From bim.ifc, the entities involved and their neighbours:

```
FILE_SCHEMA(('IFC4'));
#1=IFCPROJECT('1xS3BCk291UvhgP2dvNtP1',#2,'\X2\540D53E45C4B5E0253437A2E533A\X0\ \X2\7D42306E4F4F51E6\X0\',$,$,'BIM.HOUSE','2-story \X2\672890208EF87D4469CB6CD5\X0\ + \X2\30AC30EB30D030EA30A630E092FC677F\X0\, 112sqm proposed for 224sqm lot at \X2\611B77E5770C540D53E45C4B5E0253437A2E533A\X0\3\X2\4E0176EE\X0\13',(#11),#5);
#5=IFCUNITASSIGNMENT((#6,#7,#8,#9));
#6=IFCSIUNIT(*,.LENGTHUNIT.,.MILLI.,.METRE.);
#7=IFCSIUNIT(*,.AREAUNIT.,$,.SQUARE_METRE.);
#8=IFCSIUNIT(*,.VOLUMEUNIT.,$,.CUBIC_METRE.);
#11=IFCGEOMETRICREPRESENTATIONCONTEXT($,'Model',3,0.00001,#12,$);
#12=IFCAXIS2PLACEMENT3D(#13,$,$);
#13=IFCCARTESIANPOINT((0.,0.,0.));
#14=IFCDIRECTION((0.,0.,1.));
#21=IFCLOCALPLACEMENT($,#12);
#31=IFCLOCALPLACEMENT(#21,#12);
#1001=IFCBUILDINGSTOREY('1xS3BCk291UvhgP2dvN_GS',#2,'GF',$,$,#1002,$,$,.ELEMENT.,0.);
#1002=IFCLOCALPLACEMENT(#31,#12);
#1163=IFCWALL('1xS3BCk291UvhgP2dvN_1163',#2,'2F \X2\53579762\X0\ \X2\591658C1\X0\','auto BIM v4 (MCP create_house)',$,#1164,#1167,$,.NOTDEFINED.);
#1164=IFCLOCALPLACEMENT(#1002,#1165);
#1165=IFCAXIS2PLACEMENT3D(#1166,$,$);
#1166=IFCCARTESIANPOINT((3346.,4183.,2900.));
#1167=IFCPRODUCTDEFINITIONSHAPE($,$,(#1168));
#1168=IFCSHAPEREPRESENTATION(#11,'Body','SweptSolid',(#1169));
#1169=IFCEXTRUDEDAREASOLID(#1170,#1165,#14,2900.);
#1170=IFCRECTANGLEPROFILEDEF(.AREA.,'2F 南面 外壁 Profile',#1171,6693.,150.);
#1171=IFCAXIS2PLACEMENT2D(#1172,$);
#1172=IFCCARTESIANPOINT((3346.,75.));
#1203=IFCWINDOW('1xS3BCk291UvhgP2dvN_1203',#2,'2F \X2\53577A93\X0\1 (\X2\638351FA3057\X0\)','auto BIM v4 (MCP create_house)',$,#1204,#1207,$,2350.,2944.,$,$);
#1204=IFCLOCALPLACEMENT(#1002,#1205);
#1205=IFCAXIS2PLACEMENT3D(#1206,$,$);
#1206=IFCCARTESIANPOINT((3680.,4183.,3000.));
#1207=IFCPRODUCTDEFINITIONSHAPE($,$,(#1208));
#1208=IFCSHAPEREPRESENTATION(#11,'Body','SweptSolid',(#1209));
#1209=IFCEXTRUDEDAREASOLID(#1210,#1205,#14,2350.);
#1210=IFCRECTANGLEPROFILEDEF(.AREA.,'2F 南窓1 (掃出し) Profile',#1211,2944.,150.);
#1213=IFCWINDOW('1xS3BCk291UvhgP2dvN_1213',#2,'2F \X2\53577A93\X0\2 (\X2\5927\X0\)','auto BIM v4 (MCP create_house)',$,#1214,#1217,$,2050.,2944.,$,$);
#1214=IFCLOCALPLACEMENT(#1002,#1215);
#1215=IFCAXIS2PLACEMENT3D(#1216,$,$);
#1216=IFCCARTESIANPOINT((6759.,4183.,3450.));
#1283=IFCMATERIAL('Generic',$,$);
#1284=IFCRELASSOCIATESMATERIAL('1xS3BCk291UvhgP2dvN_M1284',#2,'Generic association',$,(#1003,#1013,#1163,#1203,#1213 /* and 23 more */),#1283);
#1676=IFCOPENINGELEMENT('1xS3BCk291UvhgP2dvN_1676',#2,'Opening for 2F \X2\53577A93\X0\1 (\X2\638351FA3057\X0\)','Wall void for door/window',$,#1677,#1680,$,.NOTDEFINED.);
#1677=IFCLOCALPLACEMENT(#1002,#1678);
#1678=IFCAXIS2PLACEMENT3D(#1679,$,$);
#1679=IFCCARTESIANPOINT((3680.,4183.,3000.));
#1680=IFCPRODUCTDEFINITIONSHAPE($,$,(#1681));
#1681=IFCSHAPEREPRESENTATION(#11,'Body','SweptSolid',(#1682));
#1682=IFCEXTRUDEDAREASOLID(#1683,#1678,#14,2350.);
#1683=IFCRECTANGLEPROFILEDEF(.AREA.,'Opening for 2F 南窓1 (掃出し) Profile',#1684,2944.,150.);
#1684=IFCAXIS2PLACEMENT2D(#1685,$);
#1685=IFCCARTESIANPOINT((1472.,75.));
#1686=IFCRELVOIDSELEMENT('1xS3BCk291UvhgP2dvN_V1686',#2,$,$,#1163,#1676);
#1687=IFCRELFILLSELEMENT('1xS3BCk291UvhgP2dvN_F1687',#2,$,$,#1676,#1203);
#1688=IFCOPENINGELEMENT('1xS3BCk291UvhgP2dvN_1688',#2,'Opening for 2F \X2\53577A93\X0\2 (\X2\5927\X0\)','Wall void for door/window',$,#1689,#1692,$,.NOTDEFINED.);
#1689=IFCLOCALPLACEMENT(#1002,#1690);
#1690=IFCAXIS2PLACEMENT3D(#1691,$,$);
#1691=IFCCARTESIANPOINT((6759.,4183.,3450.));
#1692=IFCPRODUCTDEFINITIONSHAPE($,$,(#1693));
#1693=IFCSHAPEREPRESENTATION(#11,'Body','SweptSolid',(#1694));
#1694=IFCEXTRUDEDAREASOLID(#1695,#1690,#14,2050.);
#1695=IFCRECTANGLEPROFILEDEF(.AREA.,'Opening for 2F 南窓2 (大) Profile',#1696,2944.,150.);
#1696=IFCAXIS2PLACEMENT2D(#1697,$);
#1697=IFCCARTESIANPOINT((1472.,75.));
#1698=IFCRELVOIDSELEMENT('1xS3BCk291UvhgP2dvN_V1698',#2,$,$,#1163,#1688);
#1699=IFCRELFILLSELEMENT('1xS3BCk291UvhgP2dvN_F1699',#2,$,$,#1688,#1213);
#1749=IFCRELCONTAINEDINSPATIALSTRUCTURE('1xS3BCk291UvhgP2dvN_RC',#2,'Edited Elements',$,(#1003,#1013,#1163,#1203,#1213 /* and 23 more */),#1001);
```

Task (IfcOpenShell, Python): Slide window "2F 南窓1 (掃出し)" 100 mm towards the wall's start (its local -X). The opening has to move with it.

```python
import ifcopenshell
import ifcopenshell.api.geometry
import ifcopenshell.util.placement

model = ifcopenshell.open("bim.ifc")

window = model.by_id(1203)
opening = window.FillsVoids[0].RelatingOpeningElement
wall = opening.VoidsElements[0].RelatingBuildingElement

wall_matrix = ifcopenshell.util.placement.get_local_placement(wall.ObjectPlacement)
shift = wall_matrix[:3, 0] * -100.0
before = ifcopenshell.util.placement.get_local_placement(window.ObjectPlacement)[:3, 3].copy()

# The window is not placed relative to its opening, so move both.
for product in (opening, window):
    matrix = ifcopenshell.util.placement.get_local_placement(product.ObjectPlacement)
    matrix[:3, 3] += shift
    ifcopenshell.api.geometry.edit_object_placement(model, product=product, matrix=matrix, is_si=False)

after = ifcopenshell.util.placement.get_local_placement(window.ObjectPlacement)[:3, 3]
print("window moved by", (after - before).round(3) + 0.0)

model.write("bim_edited.ifc")
```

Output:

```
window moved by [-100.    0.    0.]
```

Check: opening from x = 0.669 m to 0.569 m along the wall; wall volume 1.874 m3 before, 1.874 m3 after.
